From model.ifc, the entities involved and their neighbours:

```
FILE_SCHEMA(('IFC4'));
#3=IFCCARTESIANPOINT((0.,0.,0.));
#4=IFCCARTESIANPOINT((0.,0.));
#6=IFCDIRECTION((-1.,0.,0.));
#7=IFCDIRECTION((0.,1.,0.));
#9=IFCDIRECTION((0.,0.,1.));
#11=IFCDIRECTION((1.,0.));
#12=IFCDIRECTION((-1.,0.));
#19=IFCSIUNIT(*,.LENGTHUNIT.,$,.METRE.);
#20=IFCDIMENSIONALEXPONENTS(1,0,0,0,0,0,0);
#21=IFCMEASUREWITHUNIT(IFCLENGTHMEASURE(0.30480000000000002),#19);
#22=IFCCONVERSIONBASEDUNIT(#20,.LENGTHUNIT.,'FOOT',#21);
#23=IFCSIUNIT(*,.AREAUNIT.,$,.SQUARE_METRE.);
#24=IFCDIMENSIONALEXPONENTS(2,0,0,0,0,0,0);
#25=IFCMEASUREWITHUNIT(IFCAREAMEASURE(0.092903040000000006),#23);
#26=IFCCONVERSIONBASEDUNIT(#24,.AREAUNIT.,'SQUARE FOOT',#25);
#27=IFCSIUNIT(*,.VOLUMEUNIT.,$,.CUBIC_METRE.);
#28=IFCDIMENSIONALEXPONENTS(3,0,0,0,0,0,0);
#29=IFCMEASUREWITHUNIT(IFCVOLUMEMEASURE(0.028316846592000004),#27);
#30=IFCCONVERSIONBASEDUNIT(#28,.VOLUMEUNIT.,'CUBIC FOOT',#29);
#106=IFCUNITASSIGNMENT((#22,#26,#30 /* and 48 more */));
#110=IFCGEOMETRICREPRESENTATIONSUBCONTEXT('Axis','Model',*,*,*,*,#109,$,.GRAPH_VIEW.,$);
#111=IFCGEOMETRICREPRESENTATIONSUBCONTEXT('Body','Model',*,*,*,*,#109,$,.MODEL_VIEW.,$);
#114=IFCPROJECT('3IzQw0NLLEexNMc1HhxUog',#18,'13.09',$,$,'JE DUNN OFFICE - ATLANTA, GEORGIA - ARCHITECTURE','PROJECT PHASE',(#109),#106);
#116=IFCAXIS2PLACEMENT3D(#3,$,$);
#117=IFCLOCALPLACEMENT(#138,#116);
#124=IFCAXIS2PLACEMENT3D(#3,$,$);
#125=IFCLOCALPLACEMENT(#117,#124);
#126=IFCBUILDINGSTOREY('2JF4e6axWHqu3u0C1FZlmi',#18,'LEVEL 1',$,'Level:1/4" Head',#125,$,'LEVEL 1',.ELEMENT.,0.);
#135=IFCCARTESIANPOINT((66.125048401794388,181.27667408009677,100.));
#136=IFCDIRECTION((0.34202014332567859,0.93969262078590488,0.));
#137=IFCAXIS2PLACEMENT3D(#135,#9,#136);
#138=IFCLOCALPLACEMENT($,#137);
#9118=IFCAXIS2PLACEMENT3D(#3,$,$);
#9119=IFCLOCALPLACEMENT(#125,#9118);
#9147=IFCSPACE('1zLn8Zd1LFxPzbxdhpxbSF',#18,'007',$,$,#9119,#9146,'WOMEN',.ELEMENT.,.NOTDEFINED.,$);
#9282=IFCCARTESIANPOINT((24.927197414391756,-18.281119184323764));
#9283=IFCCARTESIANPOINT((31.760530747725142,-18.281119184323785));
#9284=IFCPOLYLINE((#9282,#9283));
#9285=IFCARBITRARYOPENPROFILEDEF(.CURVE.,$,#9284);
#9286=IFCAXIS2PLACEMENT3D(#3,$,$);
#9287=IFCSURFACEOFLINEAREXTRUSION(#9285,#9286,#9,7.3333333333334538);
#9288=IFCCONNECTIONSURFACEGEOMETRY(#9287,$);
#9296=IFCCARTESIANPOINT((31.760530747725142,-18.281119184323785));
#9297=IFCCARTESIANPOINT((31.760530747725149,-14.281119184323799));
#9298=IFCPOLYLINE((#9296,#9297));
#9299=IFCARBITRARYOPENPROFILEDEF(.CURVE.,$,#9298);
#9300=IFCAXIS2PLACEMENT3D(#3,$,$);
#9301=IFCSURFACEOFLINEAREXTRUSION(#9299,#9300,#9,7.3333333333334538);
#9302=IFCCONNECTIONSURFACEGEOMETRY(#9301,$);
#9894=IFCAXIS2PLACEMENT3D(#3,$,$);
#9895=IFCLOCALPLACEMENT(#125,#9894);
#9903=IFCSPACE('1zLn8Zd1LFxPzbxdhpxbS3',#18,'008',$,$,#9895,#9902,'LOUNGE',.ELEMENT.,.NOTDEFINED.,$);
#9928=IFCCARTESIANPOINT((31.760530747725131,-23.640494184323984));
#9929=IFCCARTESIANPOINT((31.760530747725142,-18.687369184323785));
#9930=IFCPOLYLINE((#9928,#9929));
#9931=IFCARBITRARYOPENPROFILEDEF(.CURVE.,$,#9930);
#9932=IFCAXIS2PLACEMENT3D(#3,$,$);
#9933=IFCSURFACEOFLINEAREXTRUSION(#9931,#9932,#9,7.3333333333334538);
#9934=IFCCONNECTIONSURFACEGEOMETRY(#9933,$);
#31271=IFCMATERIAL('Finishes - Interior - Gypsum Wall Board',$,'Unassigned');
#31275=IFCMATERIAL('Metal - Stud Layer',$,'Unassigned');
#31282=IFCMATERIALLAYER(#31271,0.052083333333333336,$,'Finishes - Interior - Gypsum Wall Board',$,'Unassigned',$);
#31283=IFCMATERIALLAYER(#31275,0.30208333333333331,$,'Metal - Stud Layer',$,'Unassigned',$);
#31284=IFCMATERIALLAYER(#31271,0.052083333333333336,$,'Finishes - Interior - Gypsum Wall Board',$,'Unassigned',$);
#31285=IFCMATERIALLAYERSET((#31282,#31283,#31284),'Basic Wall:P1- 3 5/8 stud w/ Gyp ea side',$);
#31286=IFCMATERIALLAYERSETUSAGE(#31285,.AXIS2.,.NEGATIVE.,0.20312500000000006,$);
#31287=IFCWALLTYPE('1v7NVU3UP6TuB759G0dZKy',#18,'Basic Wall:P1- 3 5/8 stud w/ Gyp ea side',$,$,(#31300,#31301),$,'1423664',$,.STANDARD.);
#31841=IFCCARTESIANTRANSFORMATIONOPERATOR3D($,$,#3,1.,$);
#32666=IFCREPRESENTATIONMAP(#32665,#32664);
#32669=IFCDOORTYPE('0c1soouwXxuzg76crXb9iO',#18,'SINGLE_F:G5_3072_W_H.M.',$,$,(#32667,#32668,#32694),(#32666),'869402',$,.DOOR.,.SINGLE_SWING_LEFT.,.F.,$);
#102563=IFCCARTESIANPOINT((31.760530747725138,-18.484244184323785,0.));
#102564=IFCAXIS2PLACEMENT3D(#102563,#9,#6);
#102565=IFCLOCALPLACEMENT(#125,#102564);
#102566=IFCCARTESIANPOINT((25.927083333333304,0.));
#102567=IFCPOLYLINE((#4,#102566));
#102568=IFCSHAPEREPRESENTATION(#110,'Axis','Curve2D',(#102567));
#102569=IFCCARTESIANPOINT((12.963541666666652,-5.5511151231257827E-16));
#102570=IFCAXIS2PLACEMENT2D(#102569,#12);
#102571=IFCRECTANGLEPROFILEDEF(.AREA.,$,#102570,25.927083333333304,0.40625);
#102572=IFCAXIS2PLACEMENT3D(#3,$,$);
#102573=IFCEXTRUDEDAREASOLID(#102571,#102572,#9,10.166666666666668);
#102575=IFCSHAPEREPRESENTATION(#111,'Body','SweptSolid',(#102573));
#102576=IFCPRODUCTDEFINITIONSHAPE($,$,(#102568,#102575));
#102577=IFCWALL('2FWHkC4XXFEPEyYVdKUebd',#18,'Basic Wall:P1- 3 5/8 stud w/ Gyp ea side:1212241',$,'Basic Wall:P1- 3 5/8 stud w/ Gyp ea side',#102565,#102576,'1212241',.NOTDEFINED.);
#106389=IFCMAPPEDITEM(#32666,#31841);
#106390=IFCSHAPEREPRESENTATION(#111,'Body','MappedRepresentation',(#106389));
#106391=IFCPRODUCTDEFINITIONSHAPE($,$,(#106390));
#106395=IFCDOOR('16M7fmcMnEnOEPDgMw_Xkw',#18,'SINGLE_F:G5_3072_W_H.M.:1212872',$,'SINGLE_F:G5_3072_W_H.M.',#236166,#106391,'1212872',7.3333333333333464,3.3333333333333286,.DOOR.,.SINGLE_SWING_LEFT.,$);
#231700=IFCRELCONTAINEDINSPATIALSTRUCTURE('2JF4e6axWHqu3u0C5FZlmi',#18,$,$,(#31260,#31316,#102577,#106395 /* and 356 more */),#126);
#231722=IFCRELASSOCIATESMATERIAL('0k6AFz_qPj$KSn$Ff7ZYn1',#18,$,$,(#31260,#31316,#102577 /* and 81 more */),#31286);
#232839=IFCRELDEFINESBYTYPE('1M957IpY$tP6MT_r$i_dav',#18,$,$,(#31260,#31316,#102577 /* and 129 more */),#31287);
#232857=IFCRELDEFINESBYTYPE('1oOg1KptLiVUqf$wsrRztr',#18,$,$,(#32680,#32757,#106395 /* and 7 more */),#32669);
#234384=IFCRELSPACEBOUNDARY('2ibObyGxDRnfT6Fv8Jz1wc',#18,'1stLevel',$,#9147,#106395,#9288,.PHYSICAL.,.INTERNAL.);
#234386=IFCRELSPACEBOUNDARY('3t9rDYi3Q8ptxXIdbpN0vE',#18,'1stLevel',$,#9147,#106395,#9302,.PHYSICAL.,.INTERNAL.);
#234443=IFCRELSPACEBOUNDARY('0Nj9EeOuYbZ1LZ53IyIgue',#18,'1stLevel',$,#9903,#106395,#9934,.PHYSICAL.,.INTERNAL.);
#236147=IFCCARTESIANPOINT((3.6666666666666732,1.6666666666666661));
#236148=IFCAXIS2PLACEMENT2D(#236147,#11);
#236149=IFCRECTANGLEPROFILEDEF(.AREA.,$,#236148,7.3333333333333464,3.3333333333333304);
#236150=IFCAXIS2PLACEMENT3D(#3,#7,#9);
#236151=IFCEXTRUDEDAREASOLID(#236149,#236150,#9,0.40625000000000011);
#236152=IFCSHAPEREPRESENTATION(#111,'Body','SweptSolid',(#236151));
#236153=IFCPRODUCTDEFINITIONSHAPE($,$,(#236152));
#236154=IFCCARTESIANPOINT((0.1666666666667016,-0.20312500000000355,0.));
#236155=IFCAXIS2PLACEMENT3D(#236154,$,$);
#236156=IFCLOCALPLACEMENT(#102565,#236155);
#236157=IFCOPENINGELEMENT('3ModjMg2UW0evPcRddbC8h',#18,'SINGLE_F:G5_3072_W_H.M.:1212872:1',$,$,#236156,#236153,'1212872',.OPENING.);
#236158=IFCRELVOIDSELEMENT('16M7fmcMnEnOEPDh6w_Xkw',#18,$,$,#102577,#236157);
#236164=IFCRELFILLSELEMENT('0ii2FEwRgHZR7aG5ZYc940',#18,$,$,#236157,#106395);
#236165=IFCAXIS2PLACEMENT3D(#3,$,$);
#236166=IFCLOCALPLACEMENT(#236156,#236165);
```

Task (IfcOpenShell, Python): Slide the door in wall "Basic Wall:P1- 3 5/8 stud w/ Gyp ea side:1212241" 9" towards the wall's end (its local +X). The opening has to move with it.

```python
import numpy as np
import ifcopenshell
import ifcopenshell.api.geometry
import ifcopenshell.util.placement
import ifcopenshell.util.unit

model = ifcopenshell.open("model.ifc")
unit_scale = ifcopenshell.util.unit.calculate_unit_scale(model)

door = model.by_id(106395)
opening = door.FillsVoids[0].RelatingOpeningElement
wall = opening.VoidsElements[0].RelatingBuildingElement

wall_matrix = ifcopenshell.util.placement.get_local_placement(wall.ObjectPlacement)
shift = wall_matrix[:3, 0] * 9 * 0.0254 / unit_scale
before = ifcopenshell.util.placement.get_local_placement(door.ObjectPlacement)[:3, 3].copy()

# The door is placed relative to its opening, so it follows when the opening moves.
matrix = ifcopenshell.util.placement.get_local_placement(opening.ObjectPlacement)
matrix[:3, 3] += shift
ifcopenshell.api.geometry.edit_object_placement(
    model, product=opening, matrix=matrix, is_si=False, should_transform_children=True
)

# Space boundary surfaces are stored in each space's coordinates; move them too.
for rel in door.ProvidesBoundaries:
    if not rel.ConnectionGeometry:
        continue
    surface = rel.ConnectionGeometry.SurfaceOnRelatingElement
    space_matrix = ifcopenshell.util.placement.get_local_placement(rel.RelatingSpace.ObjectPlacement)
    point = np.array(surface.Position.Location.Coordinates) + space_matrix[:3, :3].T @ shift
    surface.Position = model.createIfcAxis2Placement3D(
        model.createIfcCartesianPoint(point.tolist()), surface.Position.Axis, surface.Position.RefDirection
    )

after = ifcopenshell.util.placement.get_local_placement(door.ObjectPlacement)[:3, 3]
print("door moved by", (after - before).round(3) + 0.0)

model.write("model_edited.ifc")
```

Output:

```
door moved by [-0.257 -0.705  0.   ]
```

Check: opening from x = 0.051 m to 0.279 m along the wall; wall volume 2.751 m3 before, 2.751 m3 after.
